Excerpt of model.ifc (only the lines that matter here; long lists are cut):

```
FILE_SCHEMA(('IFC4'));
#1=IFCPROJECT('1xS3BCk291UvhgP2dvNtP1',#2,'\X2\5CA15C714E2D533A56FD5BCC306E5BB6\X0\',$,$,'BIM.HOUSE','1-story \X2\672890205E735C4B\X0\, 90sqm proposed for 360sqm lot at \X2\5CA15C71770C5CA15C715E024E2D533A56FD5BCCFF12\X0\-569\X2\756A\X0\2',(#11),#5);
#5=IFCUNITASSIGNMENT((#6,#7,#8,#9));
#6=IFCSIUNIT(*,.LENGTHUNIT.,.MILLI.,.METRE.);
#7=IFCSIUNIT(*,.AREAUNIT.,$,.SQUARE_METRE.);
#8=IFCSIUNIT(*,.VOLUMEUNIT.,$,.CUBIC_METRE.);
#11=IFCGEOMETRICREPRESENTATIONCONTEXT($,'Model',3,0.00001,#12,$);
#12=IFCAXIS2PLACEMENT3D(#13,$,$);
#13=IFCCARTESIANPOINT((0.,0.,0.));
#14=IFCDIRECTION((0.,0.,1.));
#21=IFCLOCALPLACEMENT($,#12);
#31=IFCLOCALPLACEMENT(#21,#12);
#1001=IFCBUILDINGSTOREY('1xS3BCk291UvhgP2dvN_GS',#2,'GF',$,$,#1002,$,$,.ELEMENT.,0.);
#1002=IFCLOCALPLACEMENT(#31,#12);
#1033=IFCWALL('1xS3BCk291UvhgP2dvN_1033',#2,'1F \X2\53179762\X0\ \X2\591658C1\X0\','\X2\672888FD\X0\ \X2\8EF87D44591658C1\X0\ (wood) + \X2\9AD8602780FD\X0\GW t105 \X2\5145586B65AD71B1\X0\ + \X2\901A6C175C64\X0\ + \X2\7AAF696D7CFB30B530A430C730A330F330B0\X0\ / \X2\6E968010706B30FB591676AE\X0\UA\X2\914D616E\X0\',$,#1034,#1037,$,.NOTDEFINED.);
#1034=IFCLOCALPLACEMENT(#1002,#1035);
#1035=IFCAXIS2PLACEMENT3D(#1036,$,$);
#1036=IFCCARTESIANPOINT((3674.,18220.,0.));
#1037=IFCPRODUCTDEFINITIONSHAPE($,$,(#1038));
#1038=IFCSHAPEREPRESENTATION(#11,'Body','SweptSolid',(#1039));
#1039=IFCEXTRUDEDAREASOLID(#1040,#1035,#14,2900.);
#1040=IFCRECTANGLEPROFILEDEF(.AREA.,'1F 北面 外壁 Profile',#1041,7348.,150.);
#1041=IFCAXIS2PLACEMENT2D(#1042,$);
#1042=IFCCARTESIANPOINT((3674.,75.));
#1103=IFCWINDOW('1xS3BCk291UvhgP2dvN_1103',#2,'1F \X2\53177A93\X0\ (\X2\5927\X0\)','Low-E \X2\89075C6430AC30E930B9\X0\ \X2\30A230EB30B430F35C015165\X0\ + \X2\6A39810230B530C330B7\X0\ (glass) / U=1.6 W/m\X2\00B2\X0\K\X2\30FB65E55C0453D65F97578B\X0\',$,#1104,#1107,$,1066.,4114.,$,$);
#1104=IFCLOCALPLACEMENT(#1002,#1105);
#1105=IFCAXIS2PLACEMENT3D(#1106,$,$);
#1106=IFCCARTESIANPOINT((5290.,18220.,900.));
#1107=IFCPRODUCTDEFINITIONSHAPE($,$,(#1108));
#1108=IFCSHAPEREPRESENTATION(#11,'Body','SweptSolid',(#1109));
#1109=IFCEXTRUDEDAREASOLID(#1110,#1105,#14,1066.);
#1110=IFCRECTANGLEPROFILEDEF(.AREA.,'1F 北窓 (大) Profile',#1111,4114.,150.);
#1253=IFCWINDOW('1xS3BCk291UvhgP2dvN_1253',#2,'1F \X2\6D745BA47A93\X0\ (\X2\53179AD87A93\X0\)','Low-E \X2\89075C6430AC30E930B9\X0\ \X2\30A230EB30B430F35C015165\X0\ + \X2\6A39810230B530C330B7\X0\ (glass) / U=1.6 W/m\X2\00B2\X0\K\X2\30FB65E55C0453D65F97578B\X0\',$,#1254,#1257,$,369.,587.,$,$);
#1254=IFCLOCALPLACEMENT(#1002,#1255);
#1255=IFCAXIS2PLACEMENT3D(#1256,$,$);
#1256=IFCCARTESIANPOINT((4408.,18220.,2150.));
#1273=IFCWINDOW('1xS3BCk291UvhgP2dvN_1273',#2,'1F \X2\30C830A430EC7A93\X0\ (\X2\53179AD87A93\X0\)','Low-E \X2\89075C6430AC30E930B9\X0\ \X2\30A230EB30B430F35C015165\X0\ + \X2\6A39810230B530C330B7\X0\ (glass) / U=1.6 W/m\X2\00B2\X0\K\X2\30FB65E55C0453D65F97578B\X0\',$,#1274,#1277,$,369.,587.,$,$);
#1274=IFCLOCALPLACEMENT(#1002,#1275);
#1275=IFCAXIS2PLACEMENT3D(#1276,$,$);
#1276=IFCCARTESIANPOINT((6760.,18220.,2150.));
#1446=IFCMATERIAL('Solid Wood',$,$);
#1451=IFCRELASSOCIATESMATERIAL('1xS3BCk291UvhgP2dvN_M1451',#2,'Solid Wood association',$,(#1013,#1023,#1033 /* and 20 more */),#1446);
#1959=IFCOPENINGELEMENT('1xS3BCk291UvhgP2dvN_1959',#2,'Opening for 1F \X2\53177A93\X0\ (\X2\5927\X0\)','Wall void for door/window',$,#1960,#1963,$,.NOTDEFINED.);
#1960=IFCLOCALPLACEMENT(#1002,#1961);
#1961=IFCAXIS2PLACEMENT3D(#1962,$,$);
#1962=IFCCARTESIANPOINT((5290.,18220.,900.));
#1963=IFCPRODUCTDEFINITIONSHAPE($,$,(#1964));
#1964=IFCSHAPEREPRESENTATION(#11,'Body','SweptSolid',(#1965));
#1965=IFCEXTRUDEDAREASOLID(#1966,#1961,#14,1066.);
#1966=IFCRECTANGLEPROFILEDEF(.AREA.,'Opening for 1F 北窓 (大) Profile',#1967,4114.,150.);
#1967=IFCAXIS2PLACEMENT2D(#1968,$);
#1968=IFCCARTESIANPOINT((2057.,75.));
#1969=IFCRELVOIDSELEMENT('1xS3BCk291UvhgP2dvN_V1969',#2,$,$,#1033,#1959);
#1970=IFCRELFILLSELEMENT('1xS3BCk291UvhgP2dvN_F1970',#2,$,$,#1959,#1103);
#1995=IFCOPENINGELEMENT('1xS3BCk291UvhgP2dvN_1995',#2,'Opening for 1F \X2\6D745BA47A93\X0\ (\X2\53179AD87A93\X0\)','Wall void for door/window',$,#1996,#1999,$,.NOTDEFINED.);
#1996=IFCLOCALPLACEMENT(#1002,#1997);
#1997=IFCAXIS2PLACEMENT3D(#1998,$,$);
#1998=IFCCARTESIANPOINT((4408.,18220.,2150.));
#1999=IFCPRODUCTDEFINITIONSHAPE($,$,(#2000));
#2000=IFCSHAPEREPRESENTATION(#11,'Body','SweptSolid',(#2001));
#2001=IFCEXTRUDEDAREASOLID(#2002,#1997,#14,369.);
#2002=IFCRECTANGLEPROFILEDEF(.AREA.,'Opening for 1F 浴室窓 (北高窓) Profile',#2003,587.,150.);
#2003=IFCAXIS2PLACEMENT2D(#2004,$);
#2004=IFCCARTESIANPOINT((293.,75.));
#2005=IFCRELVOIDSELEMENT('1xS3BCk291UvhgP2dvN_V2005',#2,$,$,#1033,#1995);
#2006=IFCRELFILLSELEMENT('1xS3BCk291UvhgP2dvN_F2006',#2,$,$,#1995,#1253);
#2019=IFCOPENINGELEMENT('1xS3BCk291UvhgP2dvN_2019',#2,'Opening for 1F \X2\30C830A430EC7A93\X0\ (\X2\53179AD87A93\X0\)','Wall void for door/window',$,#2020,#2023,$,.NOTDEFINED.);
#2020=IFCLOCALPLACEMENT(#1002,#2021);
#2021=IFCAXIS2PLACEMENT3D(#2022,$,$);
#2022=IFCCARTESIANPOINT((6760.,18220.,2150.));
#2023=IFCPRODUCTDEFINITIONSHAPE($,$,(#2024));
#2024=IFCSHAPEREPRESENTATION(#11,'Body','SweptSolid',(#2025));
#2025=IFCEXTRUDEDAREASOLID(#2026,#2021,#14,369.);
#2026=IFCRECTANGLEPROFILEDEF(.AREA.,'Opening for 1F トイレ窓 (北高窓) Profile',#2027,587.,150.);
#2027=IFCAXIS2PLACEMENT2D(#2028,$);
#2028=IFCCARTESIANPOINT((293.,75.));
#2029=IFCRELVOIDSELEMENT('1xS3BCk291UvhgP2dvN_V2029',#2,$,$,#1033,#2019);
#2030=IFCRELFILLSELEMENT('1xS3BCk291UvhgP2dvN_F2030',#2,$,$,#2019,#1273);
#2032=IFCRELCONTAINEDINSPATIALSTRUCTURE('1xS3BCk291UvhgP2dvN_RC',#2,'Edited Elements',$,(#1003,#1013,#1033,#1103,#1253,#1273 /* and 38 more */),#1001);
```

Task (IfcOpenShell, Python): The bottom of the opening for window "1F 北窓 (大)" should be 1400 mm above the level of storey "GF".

```python
import numpy as np
import ifcopenshell
import ifcopenshell.api.geometry
import ifcopenshell.geom
import ifcopenshell.util.element
import ifcopenshell.util.placement
import ifcopenshell.util.shape
import ifcopenshell.util.unit

model = ifcopenshell.open("model.ifc")
unit_scale = ifcopenshell.util.unit.calculate_unit_scale(model)

window = model.by_guid("1xS3BCk291UvhgP2dvN_1103")
opening = window.FillsVoids[0].RelatingOpeningElement
storey = ifcopenshell.util.element.get_container(window, ifc_class="IfcBuildingStorey")
level = ifcopenshell.util.placement.get_local_placement(storey.ObjectPlacement)[2, 3]

# The opening's origin need not be at the sill, so measure its lowest point.
shape = ifcopenshell.geom.create_shape(ifcopenshell.geom.settings(), opening)
bottom = ifcopenshell.util.shape.get_shape_bottom_elevation(shape, shape.geometry) / unit_scale
dz = level + 1.4 / unit_scale - bottom

shift = np.array([0.0, 0.0, dz])
# The window is not placed relative to its opening, so move both.
for product in (opening, window):
    matrix = ifcopenshell.util.placement.get_local_placement(product.ObjectPlacement)
    matrix[:3, 3] += shift
    ifcopenshell.api.geometry.edit_object_placement(model, product=product, matrix=matrix, is_si=False)

print(f"moved by {dz * unit_scale:+.3f} m")

model.write("model_updated.ifc")
```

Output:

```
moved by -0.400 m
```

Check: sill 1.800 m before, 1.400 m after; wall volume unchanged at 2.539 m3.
